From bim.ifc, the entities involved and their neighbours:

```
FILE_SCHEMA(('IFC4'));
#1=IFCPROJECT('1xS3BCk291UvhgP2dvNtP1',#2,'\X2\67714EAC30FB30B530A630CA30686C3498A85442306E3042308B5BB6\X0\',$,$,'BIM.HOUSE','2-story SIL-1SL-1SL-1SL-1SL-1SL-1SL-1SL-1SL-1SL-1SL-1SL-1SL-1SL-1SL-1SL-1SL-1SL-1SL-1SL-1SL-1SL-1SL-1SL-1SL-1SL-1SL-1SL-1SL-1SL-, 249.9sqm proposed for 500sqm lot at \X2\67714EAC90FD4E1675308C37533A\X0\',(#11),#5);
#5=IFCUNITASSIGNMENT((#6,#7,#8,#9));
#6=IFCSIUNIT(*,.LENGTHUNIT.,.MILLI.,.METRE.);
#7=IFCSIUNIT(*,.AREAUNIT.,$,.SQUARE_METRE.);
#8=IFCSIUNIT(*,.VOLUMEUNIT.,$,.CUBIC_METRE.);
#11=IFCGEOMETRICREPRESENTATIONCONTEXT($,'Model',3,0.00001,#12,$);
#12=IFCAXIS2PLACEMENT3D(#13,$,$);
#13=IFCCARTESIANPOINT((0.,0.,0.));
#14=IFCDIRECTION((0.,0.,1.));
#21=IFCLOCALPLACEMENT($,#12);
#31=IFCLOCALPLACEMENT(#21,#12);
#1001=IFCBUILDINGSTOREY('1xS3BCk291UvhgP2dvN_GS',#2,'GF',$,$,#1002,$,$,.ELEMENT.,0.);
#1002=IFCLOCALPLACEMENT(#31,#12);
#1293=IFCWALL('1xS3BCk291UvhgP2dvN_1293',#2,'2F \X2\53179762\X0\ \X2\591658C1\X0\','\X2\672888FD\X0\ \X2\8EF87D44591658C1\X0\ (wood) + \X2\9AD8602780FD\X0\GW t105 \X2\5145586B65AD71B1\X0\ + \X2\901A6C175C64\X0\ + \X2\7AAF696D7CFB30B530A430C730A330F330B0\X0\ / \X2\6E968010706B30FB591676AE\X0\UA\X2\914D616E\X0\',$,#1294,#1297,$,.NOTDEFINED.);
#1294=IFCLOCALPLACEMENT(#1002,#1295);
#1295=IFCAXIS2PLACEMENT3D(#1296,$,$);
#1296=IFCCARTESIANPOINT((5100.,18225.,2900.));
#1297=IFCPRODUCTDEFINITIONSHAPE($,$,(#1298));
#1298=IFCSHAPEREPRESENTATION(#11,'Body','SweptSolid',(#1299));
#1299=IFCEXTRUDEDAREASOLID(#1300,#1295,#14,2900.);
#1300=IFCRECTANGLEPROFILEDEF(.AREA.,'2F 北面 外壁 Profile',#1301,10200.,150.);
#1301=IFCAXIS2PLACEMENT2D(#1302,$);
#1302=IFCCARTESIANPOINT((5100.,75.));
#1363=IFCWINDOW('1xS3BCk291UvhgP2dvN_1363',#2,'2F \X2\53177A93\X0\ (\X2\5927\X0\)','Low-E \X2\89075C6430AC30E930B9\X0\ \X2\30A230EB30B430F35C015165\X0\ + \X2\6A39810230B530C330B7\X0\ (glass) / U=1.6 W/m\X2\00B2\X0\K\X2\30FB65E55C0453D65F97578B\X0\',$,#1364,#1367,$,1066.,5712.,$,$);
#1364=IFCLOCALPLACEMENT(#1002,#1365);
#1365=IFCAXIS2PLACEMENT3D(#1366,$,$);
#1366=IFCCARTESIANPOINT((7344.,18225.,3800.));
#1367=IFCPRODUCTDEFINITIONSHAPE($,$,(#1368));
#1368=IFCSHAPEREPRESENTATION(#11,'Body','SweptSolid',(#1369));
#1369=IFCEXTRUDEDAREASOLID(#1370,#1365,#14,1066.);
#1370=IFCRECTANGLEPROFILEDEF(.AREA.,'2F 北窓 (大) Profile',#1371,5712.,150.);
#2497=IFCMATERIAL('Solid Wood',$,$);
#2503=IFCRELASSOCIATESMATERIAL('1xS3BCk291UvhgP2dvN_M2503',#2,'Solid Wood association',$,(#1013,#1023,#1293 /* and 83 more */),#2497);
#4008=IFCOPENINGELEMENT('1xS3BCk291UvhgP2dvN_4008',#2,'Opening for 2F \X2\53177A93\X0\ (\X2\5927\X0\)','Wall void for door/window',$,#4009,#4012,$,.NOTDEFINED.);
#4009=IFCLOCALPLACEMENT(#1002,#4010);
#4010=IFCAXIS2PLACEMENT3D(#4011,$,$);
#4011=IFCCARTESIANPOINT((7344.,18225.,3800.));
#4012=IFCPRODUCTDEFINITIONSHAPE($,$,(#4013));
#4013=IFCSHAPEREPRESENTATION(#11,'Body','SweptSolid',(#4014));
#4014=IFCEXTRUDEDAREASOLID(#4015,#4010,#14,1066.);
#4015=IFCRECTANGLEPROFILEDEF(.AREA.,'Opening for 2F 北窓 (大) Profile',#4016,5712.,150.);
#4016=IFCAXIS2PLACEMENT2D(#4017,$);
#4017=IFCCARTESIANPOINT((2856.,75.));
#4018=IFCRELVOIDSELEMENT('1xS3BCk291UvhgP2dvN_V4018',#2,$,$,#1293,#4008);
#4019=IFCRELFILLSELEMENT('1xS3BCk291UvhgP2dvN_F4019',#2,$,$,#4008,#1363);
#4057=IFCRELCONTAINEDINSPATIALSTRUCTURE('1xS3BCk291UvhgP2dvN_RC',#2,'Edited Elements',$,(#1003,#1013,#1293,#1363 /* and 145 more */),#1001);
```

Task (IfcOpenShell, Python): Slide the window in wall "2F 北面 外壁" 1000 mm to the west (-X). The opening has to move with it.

```python
import ifcopenshell
import ifcopenshell.api.geometry
import ifcopenshell.util.placement
import ifcopenshell.util.unit

model = ifcopenshell.open("bim.ifc")
unit_scale = ifcopenshell.util.unit.calculate_unit_scale(model)

window = model.by_id(1363)
opening = window.FillsVoids[0].RelatingOpeningElement
wall = opening.VoidsElements[0].RelatingBuildingElement

wall_matrix = ifcopenshell.util.placement.get_local_placement(wall.ObjectPlacement)
shift = wall_matrix[:3, 0] * -1 / unit_scale
before = ifcopenshell.util.placement.get_local_placement(window.ObjectPlacement)[:3, 3].copy()

# The window is not placed relative to its opening, so move both.
for product in (opening, window):
    matrix = ifcopenshell.util.placement.get_local_placement(product.ObjectPlacement)
    matrix[:3, 3] += shift
    ifcopenshell.api.geometry.edit_object_placement(model, product=product, matrix=matrix, is_si=False)

after = ifcopenshell.util.placement.get_local_placement(window.ObjectPlacement)[:3, 3]
print("window moved by", (after - before).round(3) + 0.0)

model.write("bim_rev.ifc")
```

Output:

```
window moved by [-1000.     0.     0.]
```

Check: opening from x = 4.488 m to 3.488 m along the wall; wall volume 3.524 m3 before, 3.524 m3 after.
